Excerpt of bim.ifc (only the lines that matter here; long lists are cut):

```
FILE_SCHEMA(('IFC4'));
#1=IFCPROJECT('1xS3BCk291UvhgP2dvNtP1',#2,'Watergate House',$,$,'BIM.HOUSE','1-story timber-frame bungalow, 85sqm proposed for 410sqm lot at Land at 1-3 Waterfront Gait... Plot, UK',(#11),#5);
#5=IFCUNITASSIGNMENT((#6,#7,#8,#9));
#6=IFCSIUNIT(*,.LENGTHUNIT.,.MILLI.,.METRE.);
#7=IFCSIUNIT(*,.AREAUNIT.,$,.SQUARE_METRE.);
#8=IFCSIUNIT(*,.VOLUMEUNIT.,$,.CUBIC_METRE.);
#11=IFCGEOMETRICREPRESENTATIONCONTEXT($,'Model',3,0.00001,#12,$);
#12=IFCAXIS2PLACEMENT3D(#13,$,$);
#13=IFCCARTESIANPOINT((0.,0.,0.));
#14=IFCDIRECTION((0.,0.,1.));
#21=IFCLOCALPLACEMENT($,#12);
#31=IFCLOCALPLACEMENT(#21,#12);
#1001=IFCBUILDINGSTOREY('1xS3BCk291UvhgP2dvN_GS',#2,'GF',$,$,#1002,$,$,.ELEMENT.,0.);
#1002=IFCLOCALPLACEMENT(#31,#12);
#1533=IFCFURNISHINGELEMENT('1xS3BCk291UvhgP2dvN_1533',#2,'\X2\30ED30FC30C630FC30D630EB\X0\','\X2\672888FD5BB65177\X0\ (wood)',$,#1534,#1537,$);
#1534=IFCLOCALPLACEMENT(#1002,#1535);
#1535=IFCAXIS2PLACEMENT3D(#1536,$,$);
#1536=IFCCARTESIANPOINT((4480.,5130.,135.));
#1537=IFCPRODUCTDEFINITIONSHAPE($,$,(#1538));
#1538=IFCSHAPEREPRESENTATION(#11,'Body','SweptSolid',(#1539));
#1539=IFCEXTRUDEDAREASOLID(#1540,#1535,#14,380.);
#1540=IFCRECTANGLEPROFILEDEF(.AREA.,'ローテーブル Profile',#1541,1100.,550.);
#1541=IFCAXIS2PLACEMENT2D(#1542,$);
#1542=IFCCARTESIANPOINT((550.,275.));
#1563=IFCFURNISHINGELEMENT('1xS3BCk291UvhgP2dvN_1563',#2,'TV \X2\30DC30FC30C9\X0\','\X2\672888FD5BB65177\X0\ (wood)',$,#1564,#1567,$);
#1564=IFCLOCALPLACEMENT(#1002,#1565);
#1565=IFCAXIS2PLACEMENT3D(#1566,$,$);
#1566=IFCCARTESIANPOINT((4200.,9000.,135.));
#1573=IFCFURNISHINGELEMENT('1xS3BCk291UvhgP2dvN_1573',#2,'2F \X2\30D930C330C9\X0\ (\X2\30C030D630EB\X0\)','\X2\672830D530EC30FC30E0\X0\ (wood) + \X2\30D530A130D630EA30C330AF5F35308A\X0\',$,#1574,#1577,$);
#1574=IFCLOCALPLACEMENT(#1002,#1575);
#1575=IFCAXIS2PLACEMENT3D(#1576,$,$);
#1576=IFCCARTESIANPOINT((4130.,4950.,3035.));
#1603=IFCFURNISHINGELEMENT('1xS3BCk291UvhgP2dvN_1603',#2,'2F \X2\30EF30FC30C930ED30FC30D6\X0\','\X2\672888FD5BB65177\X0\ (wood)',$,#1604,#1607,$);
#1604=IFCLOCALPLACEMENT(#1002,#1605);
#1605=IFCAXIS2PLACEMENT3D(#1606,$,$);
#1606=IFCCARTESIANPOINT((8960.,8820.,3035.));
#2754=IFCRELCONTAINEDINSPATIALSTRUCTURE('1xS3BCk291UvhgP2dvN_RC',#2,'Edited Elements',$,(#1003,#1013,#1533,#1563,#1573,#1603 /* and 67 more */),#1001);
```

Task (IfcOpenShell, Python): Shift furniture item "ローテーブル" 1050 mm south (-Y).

```python
import ifcopenshell
import ifcopenshell.api.geometry
import ifcopenshell.util.placement
import ifcopenshell.util.unit

model = ifcopenshell.open("bim.ifc")
unit_scale = ifcopenshell.util.unit.calculate_unit_scale(model)

item = model.by_guid("1xS3BCk291UvhgP2dvN_1533")
matrix = ifcopenshell.util.placement.get_local_placement(item.ObjectPlacement)
matrix[1, 3] -= 1.05 / unit_scale
ifcopenshell.api.geometry.edit_object_placement(model, product=item, matrix=matrix, is_si=False)

print(ifcopenshell.util.placement.get_local_placement(item.ObjectPlacement).round(3) + 0.0)

model.write("bim_edited.ifc")
```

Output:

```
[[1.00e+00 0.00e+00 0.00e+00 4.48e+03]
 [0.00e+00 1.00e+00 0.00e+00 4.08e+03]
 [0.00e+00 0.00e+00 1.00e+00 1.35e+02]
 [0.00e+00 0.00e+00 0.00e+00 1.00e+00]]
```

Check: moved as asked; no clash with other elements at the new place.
